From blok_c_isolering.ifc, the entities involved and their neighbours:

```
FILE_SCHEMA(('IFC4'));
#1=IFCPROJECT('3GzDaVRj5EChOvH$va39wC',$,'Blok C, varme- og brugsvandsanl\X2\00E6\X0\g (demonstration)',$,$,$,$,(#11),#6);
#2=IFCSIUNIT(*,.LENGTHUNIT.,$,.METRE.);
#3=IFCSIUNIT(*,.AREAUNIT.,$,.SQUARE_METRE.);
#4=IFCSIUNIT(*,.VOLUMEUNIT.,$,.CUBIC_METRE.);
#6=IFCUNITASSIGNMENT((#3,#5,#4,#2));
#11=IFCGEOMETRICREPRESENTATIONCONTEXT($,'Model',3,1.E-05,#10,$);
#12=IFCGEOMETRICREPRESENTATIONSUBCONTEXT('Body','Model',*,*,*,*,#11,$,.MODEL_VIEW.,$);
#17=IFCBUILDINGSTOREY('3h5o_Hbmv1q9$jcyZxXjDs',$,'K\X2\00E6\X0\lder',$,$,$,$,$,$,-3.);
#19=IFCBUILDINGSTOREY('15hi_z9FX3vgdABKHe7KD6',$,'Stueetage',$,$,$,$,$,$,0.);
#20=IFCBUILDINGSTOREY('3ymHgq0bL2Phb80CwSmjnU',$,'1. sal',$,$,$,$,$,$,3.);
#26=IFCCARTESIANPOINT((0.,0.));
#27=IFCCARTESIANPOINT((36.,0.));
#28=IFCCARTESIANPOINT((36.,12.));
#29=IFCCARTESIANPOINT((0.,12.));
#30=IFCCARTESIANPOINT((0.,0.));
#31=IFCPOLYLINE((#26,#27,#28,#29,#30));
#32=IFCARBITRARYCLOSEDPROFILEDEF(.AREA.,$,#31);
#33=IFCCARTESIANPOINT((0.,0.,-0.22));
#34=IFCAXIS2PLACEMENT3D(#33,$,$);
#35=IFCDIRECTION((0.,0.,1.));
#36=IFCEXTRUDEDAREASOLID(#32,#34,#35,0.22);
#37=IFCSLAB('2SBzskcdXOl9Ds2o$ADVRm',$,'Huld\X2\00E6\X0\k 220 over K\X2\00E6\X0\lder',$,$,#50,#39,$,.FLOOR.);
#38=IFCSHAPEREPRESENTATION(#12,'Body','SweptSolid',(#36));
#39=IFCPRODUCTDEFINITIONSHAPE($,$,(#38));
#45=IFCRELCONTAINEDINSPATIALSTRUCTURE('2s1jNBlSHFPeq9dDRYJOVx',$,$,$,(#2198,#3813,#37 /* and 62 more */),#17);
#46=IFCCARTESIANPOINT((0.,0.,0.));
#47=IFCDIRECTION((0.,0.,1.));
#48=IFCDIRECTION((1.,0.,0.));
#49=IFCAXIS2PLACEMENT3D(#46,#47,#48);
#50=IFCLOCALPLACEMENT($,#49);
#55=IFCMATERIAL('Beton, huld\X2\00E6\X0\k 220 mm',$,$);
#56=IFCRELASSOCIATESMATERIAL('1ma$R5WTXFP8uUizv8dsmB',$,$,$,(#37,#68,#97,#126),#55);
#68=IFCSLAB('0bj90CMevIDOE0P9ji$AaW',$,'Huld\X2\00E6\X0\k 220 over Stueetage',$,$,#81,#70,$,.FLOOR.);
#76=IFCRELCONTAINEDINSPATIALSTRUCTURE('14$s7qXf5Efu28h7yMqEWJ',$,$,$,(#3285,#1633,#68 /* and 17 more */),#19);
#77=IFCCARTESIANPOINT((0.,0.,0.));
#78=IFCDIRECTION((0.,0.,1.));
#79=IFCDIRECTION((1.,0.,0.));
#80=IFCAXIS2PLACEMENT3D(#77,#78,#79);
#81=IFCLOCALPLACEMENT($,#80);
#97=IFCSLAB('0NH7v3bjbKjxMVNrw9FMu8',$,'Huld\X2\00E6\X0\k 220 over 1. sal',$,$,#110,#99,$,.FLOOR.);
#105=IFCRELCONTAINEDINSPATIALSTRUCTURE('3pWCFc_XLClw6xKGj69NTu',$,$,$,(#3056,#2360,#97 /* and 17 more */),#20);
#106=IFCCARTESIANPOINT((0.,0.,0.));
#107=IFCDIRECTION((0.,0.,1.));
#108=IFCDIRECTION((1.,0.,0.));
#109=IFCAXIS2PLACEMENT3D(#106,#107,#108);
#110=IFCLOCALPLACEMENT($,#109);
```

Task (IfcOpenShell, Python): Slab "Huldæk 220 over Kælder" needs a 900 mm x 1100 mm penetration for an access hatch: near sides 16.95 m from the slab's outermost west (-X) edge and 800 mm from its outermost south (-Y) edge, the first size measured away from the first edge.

```python
import numpy as np
import ifcopenshell
import ifcopenshell.api.feature
import ifcopenshell.api.geometry
import ifcopenshell.api.root
import ifcopenshell.geom
import ifcopenshell.util.placement
import ifcopenshell.util.representation
import ifcopenshell.util.shape
import ifcopenshell.util.unit

model = ifcopenshell.open("blok_c_isolering.ifc")
unit_scale = ifcopenshell.util.unit.calculate_unit_scale(model)
settings = ifcopenshell.geom.settings()


def volume(element):
    """Net volume in cubic metres, openings subtracted."""
    shape = ifcopenshell.geom.create_shape(settings, element)
    return ifcopenshell.util.shape.get_volume(shape.geometry)


slab = model.by_guid("2SBzskcdXOl9Ds2o$ADVRm")
before = volume(slab)

# Extent in the slab's own axes, in metres. The edges named are its -X and -Y sides.
slab_shape = ifcopenshell.geom.create_shape(settings, slab)
vertices = ifcopenshell.util.shape.get_vertices(slab_shape.geometry)
x_min, y_min, bottom = vertices.min(axis=0)
top = vertices[:, 2].max()

opening = ifcopenshell.api.root.create_entity(model, ifc_class="IfcOpeningElement", name="Access hatch opening", predefined_type="OPENING")
context = ifcopenshell.util.representation.get_context(model, "Model", "Body", "MODEL_VIEW")
width, depth = 0.9, 1.1
outline = [(0.0, 0.0), (width, 0.0), (width, depth), (0.0, depth), (0.0, 0.0)]
# Overshoot both faces by 50 mm so the cut is clean.
shape = ifcopenshell.api.geometry.add_slab_representation(
    model, context=context, depth=top - bottom + 0.1, polyline=outline
)
ifcopenshell.api.geometry.assign_representation(model, product=opening, representation=shape)

matrix = ifcopenshell.util.placement.get_local_placement(slab.ObjectPlacement)
matrix[:, 3] = matrix @ np.append(np.array([x_min + 16.95, y_min + 0.8, bottom - 0.05]) / unit_scale, 1.0)
ifcopenshell.api.geometry.edit_object_placement(model, product=opening, matrix=matrix, is_si=False)
ifcopenshell.api.feature.add_feature(model, feature=opening, element=slab)

after = volume(slab)

print(f"slab volume {before:.3f} -> {after:.3f} m3")

model.write("blok_c_isolering_updated.ifc")
```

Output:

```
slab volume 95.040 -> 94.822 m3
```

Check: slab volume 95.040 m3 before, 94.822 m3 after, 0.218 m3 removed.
